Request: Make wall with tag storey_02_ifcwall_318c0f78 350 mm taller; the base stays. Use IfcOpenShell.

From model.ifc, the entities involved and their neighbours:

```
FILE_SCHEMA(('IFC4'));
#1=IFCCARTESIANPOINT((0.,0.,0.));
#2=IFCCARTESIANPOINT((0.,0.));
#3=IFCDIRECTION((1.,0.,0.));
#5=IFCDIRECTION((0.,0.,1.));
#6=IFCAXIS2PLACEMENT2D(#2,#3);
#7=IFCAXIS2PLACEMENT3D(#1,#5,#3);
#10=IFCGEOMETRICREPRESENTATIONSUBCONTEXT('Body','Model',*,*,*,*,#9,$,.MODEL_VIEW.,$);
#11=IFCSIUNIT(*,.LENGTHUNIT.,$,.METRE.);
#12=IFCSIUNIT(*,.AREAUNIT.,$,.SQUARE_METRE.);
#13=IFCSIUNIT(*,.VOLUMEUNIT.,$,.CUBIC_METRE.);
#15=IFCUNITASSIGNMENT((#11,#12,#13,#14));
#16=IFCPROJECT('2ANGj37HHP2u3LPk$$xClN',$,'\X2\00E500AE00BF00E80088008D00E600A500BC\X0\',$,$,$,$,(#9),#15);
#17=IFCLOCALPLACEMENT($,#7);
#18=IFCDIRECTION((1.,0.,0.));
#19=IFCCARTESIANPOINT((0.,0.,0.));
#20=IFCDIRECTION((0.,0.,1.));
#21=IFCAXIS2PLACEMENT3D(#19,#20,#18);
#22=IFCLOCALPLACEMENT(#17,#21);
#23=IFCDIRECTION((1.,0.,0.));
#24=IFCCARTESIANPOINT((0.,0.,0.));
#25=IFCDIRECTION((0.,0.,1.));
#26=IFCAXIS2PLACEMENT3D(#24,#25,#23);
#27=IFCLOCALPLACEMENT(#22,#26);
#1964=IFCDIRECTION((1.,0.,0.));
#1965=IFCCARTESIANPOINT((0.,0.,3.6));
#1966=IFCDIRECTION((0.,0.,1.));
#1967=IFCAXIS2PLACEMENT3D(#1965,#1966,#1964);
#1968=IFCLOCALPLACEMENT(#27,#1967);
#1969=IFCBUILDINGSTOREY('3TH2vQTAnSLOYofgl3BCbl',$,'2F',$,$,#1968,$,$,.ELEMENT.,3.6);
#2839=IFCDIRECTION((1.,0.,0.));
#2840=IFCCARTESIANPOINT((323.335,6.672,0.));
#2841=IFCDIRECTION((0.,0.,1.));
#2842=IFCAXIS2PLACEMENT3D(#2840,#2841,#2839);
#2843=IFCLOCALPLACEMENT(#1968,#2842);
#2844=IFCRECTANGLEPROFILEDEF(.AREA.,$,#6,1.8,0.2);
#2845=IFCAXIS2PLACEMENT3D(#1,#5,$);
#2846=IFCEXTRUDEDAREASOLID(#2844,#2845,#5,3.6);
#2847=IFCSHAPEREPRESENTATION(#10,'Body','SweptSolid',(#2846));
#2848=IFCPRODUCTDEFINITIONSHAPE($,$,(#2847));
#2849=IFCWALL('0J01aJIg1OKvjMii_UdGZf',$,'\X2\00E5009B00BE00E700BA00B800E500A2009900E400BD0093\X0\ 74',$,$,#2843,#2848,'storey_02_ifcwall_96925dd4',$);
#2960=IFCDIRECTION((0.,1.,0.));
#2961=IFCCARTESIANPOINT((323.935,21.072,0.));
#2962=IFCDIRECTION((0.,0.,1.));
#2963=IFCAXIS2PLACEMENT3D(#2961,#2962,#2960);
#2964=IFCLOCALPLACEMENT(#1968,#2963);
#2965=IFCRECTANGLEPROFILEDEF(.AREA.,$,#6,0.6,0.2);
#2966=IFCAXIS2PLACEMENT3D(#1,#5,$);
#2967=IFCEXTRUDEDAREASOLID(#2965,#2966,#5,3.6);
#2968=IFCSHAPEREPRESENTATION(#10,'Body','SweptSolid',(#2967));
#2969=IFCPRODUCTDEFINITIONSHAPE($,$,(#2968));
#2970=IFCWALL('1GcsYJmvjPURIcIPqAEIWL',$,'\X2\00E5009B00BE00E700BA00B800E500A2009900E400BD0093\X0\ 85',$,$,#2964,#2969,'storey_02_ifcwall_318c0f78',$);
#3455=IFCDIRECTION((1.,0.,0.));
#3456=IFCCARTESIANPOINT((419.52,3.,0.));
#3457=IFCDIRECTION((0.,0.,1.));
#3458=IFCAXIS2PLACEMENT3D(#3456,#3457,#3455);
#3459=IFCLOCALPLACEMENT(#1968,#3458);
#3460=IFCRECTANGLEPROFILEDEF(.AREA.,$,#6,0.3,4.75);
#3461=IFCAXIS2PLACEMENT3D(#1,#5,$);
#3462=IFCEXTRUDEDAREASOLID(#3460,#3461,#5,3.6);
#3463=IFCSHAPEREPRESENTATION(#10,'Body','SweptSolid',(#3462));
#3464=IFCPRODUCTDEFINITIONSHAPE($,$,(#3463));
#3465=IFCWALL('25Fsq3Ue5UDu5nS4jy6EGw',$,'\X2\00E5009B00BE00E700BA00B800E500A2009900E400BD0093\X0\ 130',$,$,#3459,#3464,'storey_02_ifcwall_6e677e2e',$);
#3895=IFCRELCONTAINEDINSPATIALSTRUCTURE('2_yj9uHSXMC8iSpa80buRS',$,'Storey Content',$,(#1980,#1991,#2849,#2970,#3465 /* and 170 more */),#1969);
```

```python
import ifcopenshell
import ifcopenshell.geom
import ifcopenshell.util.representation
import ifcopenshell.util.shape
import ifcopenshell.util.unit

model = ifcopenshell.open("model.ifc")
unit_scale = ifcopenshell.util.unit.calculate_unit_scale(model)
settings = ifcopenshell.geom.settings()


def volume(element):
    """Net volume in cubic metres, openings subtracted."""
    shape = ifcopenshell.geom.create_shape(settings, element)
    return ifcopenshell.util.shape.get_volume(shape.geometry)


wall = model.by_guid("1GcsYJmvjPURIcIPqAEIWL")
before = volume(wall)

body = ifcopenshell.util.representation.get_representation(wall, "Model", "Body")
solid = body.Items[0]
old_height = solid.Depth
solid.Depth += 0.35 / unit_scale
after = volume(wall)

print(f"height {old_height:g} -> {solid.Depth:g}, volume {before:.3f} -> {after:.3f} m3")

model.write("model_rev.ifc")
```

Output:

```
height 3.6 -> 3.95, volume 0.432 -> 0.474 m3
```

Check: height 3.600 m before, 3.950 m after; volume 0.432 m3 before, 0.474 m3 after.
